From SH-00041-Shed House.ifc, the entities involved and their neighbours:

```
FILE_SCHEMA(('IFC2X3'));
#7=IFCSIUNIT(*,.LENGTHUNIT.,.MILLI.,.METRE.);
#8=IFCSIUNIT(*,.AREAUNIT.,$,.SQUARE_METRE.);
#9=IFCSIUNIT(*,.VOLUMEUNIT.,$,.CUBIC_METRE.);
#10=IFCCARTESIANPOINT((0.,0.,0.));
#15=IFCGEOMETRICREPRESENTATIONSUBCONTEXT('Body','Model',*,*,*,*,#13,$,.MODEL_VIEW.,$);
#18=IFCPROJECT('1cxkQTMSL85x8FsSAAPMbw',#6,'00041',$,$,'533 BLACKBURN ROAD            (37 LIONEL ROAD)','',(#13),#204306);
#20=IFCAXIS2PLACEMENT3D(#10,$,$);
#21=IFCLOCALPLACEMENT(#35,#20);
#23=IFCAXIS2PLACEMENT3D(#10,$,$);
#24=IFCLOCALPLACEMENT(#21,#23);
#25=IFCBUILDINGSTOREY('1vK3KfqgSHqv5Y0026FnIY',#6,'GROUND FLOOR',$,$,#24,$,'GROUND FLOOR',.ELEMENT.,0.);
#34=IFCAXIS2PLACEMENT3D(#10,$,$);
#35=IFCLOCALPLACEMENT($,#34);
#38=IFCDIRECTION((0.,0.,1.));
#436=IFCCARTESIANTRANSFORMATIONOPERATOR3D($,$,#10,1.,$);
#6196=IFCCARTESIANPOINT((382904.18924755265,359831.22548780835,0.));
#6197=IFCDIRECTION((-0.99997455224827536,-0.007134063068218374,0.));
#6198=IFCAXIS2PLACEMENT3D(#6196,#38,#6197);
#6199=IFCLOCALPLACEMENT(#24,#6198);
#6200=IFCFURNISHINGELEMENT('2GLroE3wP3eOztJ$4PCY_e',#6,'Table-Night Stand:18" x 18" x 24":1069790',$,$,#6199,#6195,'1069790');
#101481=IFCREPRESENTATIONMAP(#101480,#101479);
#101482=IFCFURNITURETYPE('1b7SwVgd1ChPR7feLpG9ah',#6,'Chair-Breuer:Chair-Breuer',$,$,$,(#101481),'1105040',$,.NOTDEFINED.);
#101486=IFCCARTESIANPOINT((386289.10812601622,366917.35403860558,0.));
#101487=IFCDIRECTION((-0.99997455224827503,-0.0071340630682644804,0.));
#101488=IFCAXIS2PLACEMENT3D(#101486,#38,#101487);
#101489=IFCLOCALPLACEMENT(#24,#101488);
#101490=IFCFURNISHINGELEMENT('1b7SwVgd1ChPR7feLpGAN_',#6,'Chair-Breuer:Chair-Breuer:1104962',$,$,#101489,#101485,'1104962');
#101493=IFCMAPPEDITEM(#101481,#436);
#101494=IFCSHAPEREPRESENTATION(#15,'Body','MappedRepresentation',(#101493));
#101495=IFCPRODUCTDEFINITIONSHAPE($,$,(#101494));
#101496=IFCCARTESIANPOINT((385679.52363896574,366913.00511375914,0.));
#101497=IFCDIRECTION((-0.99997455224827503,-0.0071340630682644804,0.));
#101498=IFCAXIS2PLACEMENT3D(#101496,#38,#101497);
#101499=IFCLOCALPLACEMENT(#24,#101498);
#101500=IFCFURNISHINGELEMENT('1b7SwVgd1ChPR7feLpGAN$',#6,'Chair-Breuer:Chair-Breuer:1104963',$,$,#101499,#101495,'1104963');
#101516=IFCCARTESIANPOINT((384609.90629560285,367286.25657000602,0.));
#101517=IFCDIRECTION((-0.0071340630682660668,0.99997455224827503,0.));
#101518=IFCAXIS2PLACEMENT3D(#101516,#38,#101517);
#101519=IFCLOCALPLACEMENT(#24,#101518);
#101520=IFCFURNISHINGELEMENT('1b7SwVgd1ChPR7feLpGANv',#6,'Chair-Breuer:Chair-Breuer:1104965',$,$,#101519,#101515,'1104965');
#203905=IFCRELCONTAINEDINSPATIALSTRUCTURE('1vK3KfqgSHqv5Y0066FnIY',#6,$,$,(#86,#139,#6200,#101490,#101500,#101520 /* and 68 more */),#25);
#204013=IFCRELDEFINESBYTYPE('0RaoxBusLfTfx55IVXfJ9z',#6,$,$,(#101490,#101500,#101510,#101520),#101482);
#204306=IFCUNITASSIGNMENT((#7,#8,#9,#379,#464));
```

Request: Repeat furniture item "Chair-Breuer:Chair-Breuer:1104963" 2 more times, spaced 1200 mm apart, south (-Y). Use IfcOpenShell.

```python
import numpy as np
import ifcopenshell
import ifcopenshell.api.geometry
import ifcopenshell.api.root
import ifcopenshell.util.element
import ifcopenshell.util.placement
import ifcopenshell.util.unit

model = ifcopenshell.open("SH-00041-Shed House.ifc")
unit_scale = ifcopenshell.util.unit.calculate_unit_scale(model)


def reuse_history(source, copy):
    """copy_class also copies each property set's owner history, people and application; keep the originals."""
    for rel in copy.IsDefinedBy:
        if rel.is_a("IfcRelDefinesByProperties") and (history := rel.RelatingPropertyDefinition.OwnerHistory):
            rel.RelatingPropertyDefinition.OwnerHistory = source.OwnerHistory
            ifcopenshell.util.element.remove_deep2(model, history)


source = model.by_guid("1b7SwVgd1ChPR7feLpGAN$")
base = ifcopenshell.util.placement.get_local_placement(source.ObjectPlacement)
step = np.array([0.0, -1.0, 0.0]) * 1.2 / unit_scale

for i in range(1, 3):
    copy = ifcopenshell.api.root.copy_class(model, product=source)
    copy.Representation = ifcopenshell.util.element.copy_deep(
        model, source.Representation, exclude=["IfcGeometricRepresentationContext", "IfcRepresentationMap"]
    )
    copy.Name = "Chair-Breuer:Chair-Breuer"
    copy.Tag = None
    reuse_history(source, copy)
    matrix = base.copy()
    matrix[:3, 3] += i * step
    print("added at", matrix[:3, 3].round(3) + 0.0)
    ifcopenshell.api.geometry.edit_object_placement(model, product=copy, matrix=matrix, is_si=False)

model.write("SH-00041-Shed House_updated.ifc")
```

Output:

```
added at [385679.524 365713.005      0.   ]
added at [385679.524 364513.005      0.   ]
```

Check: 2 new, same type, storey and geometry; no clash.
